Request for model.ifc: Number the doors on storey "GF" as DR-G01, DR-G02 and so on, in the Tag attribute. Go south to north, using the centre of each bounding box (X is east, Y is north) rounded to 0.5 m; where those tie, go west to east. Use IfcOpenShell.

First a look at what the model holds.

```python
import ifcopenshell
import ifcopenshell.util.element
import ifcopenshell.util.placement

model = ifcopenshell.open("model.ifc")
print(model.schema)
storey = next(s for s in model.by_type("IfcBuildingStorey") if s.Name == "GF")
doors = [e for e in ifcopenshell.util.element.get_decomposition(storey) if e.is_a("IfcDoor")]
for e in sorted(doors, key=lambda e: e.id()):
    origin = ifcopenshell.util.placement.get_local_placement(e.ObjectPlacement)[:3, 3]
    print(e.id(), e.Tag, e.Name, origin.round(2) + 0.0, sep=" | ")
```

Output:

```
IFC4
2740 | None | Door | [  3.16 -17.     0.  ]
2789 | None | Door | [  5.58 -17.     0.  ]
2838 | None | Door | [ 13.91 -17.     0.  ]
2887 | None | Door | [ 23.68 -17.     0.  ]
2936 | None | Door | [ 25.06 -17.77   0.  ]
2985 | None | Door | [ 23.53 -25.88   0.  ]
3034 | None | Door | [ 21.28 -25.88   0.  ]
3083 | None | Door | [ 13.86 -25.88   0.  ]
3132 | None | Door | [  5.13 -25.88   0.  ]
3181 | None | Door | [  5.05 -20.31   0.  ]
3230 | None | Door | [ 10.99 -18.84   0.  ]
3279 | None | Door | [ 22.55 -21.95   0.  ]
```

```python
import ifcopenshell
import ifcopenshell.geom
import ifcopenshell.util.element
import ifcopenshell.util.shape

model = ifcopenshell.open("model.ifc")
settings = ifcopenshell.geom.settings()
settings.set("use-world-coords", True)


def centre(element):
    shape = ifcopenshell.geom.create_shape(settings, element)
    return ifcopenshell.util.shape.get_bbox_centroid(shape.geometry)


storey = next(s for s in model.by_type("IfcBuildingStorey") if s.Name == "GF")
doors = [e for e in ifcopenshell.util.element.get_decomposition(storey) if e.is_a("IfcDoor")]

# Insertion points can sit at a corner or the storey origin, so sort by the geometry (in metres).
centres = {e: centre(e) for e in doors}
doors.sort(key=lambda e: (round(centres[e][1] / 0.5), centres[e][0]))

for i, e in enumerate(doors, start=1):
    number = f"DR-G{i:02d}"
    e.Tag = number
    print(e.id(), number)

model.write("model_v2.ifc")
```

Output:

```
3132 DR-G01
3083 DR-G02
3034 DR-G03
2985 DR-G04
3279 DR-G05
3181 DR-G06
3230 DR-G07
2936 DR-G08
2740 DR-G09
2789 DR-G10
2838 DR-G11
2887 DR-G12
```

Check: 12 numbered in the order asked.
